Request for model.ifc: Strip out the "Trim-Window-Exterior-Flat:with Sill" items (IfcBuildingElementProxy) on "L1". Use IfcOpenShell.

First a look at what the model holds.

```python
import ifcopenshell
import ifcopenshell.util.element

model = ifcopenshell.open("model.ifc")
print(model.schema)
storey = next(s for s in model.by_type("IfcBuildingStorey") if s.Name == "L1")
proxies = [e for e in ifcopenshell.util.element.get_decomposition(storey) if e.is_a("IfcBuildingElementProxy")]
seen = {}
for e in proxies:
    element_type = ifcopenshell.util.element.get_type(e)
    name = element_type.Name if element_type not in (None, e) else None
    seen[name] = seen.get(name, 0) + 1
for name, count in sorted(seen.items(), key=str):
    print(count, "x", name)
```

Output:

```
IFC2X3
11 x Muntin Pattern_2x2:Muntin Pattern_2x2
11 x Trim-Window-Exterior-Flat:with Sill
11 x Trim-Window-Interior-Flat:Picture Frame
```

```python
import ifcopenshell
import ifcopenshell.api.root
import ifcopenshell.util.element

model = ifcopenshell.open("model.ifc")

storey = next(s for s in model.by_type("IfcBuildingStorey") if s.Name == "L1")
proxies = [e for e in ifcopenshell.util.element.get_decomposition(storey) if e.is_a("IfcBuildingElementProxy")]
targets = [e for e in proxies if (t := ifcopenshell.util.element.get_type(e)) not in (None, e) and t.Name == "Trim-Window-Exterior-Flat:with Sill"]

for e in targets:
    ifcopenshell.api.root.remove_product(model, product=e)
print(len(targets), "removed")

model.write("model_rev.ifc")
```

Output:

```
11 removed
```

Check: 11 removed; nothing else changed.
